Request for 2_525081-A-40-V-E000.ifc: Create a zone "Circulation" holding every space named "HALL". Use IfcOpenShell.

First a look at what the model holds.

```python
import ifcopenshell

model = ifcopenshell.open("2_525081-A-40-V-E000.ifc")
print(model.schema)
seen = {}
for space in model.by_type("IfcSpace"):
    seen[space.LongName] = seen.get(space.LongName, 0) + 1
for name, count in sorted(seen.items(), key=str):
    print(count, "x", name)
print("zones:", [z.Name for z in model.by_type("IfcZone")][:20])
```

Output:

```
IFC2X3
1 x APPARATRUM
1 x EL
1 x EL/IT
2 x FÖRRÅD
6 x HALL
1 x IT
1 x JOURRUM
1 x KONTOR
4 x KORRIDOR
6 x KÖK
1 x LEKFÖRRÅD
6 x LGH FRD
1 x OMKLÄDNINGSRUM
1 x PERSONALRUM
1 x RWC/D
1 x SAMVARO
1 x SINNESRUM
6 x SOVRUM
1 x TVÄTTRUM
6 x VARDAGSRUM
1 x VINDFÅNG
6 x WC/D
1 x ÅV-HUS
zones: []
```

```python
import ifcopenshell
import ifcopenshell.api.group
import ifcopenshell.api.root

model = ifcopenshell.open("2_525081-A-40-V-E000.ifc")

names = {"HALL"}
spaces = [s for s in model.by_type("IfcSpace") if s.LongName in names]

zone = ifcopenshell.api.root.create_entity(model, ifc_class="IfcZone", name="Circulation")
ifcopenshell.api.group.assign_group(model, products=spaces, group=zone)
print(len(spaces), "spaces in", zone.Name)

model.write("2_525081-A-40-V-E000_updated.ifc")
```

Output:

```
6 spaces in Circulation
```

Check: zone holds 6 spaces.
